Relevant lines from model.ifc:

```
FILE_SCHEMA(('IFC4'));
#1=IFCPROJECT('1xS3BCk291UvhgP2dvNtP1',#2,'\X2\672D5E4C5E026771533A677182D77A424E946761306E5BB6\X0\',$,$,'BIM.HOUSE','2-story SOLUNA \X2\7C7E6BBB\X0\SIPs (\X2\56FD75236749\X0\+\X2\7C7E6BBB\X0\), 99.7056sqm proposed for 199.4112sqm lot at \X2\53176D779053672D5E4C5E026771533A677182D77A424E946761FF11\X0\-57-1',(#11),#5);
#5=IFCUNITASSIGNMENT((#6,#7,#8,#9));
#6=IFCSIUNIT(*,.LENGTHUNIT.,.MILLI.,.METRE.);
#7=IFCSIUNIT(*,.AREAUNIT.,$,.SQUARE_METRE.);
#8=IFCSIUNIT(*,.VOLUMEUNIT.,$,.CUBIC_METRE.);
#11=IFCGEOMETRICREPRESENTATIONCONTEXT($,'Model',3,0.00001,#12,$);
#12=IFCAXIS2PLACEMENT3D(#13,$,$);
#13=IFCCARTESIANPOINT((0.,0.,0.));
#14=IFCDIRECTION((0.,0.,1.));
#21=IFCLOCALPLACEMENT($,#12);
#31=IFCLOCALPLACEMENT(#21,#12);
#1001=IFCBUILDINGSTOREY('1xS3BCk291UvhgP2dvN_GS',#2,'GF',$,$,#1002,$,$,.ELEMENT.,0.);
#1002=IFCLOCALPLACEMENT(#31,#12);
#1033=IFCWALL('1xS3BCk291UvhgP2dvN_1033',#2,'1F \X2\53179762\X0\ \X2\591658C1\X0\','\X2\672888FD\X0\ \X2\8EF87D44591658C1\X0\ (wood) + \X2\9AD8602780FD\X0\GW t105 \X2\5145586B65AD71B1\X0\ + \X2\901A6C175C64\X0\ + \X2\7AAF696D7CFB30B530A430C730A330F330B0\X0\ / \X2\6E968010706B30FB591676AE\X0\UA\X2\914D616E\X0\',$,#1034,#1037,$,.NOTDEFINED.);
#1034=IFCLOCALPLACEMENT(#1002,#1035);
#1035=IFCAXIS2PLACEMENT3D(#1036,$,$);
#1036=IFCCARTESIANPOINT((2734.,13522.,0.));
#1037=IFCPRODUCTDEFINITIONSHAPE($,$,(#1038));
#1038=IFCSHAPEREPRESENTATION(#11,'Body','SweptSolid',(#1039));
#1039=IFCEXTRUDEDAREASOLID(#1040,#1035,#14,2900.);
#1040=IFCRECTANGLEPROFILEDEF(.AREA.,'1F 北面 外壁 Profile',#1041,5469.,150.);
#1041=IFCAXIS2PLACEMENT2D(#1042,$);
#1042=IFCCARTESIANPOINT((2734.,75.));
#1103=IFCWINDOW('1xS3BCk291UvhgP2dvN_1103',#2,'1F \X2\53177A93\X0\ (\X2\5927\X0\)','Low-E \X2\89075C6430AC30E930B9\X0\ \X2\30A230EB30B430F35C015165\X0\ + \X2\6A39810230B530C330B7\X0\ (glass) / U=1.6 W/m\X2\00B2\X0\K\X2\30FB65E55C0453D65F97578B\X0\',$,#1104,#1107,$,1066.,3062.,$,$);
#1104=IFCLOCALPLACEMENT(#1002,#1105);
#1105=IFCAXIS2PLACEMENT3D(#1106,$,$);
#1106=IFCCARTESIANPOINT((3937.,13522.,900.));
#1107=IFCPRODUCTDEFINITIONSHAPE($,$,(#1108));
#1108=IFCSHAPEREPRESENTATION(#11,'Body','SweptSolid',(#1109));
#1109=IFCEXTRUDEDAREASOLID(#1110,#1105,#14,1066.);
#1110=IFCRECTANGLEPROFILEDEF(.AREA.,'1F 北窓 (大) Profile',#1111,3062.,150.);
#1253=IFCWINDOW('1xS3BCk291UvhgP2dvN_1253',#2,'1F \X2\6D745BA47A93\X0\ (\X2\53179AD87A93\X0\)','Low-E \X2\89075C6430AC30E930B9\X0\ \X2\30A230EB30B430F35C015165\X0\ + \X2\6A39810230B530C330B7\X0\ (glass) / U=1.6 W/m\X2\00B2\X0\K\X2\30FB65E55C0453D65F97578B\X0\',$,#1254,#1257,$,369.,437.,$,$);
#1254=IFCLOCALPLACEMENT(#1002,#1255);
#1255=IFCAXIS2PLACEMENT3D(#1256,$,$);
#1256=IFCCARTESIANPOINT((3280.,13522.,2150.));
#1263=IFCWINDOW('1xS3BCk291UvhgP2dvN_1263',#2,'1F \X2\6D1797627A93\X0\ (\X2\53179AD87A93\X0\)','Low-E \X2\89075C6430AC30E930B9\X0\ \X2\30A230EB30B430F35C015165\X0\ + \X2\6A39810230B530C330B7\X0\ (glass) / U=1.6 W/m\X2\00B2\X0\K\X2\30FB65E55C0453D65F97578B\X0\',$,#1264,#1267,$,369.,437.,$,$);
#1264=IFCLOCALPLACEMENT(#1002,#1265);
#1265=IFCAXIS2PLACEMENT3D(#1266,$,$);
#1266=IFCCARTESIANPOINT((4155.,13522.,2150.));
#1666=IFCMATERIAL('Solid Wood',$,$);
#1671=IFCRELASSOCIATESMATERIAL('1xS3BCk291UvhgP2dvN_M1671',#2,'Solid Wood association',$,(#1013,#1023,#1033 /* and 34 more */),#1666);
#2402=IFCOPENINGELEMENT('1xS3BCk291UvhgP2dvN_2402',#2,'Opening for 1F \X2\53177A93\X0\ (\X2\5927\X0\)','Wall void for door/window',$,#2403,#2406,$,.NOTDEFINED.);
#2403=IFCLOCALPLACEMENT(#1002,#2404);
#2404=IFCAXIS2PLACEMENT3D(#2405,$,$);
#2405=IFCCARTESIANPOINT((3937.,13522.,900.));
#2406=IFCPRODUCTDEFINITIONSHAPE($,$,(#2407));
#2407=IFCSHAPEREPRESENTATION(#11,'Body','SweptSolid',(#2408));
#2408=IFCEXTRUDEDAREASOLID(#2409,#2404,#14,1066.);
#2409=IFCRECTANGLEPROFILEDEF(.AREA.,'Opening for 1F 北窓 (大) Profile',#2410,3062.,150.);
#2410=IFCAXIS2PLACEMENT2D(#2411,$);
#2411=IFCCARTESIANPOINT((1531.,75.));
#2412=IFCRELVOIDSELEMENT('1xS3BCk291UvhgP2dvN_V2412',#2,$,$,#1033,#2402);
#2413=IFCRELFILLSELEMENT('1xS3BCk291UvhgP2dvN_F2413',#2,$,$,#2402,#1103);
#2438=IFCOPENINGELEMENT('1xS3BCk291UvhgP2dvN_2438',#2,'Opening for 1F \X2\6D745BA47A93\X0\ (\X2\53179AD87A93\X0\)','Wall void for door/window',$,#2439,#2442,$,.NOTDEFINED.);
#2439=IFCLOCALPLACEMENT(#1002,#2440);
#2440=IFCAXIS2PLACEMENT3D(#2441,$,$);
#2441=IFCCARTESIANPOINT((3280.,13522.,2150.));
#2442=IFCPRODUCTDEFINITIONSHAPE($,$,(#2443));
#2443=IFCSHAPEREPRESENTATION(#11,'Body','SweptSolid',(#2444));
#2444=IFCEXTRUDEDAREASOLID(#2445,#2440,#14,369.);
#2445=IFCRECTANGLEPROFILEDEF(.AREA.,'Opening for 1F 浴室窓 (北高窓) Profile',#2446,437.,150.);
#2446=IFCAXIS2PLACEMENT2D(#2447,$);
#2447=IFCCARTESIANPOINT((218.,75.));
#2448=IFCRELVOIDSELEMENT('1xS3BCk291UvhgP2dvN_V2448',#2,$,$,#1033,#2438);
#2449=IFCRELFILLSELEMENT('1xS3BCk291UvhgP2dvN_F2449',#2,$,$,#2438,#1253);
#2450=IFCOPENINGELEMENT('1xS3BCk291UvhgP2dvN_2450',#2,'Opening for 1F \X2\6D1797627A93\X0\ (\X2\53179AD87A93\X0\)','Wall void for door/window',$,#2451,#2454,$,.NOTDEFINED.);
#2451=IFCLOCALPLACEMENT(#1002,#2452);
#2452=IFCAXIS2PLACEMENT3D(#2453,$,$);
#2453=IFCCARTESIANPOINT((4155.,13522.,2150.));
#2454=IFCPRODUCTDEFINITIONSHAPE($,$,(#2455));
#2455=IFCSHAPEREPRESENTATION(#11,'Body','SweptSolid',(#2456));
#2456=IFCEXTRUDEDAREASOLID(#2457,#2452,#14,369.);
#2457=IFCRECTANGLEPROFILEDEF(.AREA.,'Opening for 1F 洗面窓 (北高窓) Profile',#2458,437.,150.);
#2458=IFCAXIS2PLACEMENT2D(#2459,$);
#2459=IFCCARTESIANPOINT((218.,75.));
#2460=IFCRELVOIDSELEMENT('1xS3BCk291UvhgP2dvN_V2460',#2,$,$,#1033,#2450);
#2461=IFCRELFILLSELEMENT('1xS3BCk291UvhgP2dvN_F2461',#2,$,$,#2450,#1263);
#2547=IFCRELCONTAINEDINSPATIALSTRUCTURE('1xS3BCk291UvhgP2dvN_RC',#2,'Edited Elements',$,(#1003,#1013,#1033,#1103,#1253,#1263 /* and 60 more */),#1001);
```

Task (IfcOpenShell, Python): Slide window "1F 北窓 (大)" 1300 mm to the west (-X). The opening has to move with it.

```python
import ifcopenshell
import ifcopenshell.api.geometry
import ifcopenshell.util.placement

model = ifcopenshell.open("model.ifc")

window = model.by_guid("1xS3BCk291UvhgP2dvN_1103")
opening = window.FillsVoids[0].RelatingOpeningElement
wall = opening.VoidsElements[0].RelatingBuildingElement

wall_matrix = ifcopenshell.util.placement.get_local_placement(wall.ObjectPlacement)
shift = wall_matrix[:3, 0] * -1300.0
before = ifcopenshell.util.placement.get_local_placement(window.ObjectPlacement)[:3, 3].copy()

# The window is not placed relative to its opening, so move both.
for product in (opening, window):
    matrix = ifcopenshell.util.placement.get_local_placement(product.ObjectPlacement)
    matrix[:3, 3] += shift
    ifcopenshell.api.geometry.edit_object_placement(model, product=product, matrix=matrix, is_si=False)

after = ifcopenshell.util.placement.get_local_placement(window.ObjectPlacement)[:3, 3]
print("window moved by", (after - before).round(3) + 0.0)

model.write("model_updated.ifc")
```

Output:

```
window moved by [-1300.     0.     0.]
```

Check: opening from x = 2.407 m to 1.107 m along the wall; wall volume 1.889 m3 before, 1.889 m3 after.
